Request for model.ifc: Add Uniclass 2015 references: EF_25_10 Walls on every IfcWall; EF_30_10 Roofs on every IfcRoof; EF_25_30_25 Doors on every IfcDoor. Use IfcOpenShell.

First a look at what the model holds.

```python
import ifcopenshell

model = ifcopenshell.open("model.ifc")
print(model.schema)
print("classifications:", [c.Name for c in model.by_type("IfcClassification")])
for ifc_class in ("IfcDoor", "IfcRoof", "IfcStair", "IfcWall", "IfcWindow"):
    print(ifc_class, len(model.by_type(ifc_class)))
```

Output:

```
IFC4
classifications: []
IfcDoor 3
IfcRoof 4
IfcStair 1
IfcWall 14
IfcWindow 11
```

```python
import ifcopenshell
import ifcopenshell.api.classification

model = ifcopenshell.open("model.ifc")

system = ifcopenshell.api.classification.add_classification(model, classification="Uniclass 2015")

codes = {
    "IfcWall": ("EF_25_10", "Walls"),
    "IfcRoof": ("EF_30_10", "Roofs"),
    "IfcDoor": ("EF_25_30_25", "Doors"),
}
for ifc_class, (code, name) in codes.items():
    products = model.by_type(ifc_class)
    ifcopenshell.api.classification.add_reference(
        model, products=products, classification=system, identification=code, name=name
    )
    print(code, len(products))

model.write("model_updated.ifc")
```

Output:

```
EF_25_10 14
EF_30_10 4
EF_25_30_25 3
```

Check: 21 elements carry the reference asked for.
